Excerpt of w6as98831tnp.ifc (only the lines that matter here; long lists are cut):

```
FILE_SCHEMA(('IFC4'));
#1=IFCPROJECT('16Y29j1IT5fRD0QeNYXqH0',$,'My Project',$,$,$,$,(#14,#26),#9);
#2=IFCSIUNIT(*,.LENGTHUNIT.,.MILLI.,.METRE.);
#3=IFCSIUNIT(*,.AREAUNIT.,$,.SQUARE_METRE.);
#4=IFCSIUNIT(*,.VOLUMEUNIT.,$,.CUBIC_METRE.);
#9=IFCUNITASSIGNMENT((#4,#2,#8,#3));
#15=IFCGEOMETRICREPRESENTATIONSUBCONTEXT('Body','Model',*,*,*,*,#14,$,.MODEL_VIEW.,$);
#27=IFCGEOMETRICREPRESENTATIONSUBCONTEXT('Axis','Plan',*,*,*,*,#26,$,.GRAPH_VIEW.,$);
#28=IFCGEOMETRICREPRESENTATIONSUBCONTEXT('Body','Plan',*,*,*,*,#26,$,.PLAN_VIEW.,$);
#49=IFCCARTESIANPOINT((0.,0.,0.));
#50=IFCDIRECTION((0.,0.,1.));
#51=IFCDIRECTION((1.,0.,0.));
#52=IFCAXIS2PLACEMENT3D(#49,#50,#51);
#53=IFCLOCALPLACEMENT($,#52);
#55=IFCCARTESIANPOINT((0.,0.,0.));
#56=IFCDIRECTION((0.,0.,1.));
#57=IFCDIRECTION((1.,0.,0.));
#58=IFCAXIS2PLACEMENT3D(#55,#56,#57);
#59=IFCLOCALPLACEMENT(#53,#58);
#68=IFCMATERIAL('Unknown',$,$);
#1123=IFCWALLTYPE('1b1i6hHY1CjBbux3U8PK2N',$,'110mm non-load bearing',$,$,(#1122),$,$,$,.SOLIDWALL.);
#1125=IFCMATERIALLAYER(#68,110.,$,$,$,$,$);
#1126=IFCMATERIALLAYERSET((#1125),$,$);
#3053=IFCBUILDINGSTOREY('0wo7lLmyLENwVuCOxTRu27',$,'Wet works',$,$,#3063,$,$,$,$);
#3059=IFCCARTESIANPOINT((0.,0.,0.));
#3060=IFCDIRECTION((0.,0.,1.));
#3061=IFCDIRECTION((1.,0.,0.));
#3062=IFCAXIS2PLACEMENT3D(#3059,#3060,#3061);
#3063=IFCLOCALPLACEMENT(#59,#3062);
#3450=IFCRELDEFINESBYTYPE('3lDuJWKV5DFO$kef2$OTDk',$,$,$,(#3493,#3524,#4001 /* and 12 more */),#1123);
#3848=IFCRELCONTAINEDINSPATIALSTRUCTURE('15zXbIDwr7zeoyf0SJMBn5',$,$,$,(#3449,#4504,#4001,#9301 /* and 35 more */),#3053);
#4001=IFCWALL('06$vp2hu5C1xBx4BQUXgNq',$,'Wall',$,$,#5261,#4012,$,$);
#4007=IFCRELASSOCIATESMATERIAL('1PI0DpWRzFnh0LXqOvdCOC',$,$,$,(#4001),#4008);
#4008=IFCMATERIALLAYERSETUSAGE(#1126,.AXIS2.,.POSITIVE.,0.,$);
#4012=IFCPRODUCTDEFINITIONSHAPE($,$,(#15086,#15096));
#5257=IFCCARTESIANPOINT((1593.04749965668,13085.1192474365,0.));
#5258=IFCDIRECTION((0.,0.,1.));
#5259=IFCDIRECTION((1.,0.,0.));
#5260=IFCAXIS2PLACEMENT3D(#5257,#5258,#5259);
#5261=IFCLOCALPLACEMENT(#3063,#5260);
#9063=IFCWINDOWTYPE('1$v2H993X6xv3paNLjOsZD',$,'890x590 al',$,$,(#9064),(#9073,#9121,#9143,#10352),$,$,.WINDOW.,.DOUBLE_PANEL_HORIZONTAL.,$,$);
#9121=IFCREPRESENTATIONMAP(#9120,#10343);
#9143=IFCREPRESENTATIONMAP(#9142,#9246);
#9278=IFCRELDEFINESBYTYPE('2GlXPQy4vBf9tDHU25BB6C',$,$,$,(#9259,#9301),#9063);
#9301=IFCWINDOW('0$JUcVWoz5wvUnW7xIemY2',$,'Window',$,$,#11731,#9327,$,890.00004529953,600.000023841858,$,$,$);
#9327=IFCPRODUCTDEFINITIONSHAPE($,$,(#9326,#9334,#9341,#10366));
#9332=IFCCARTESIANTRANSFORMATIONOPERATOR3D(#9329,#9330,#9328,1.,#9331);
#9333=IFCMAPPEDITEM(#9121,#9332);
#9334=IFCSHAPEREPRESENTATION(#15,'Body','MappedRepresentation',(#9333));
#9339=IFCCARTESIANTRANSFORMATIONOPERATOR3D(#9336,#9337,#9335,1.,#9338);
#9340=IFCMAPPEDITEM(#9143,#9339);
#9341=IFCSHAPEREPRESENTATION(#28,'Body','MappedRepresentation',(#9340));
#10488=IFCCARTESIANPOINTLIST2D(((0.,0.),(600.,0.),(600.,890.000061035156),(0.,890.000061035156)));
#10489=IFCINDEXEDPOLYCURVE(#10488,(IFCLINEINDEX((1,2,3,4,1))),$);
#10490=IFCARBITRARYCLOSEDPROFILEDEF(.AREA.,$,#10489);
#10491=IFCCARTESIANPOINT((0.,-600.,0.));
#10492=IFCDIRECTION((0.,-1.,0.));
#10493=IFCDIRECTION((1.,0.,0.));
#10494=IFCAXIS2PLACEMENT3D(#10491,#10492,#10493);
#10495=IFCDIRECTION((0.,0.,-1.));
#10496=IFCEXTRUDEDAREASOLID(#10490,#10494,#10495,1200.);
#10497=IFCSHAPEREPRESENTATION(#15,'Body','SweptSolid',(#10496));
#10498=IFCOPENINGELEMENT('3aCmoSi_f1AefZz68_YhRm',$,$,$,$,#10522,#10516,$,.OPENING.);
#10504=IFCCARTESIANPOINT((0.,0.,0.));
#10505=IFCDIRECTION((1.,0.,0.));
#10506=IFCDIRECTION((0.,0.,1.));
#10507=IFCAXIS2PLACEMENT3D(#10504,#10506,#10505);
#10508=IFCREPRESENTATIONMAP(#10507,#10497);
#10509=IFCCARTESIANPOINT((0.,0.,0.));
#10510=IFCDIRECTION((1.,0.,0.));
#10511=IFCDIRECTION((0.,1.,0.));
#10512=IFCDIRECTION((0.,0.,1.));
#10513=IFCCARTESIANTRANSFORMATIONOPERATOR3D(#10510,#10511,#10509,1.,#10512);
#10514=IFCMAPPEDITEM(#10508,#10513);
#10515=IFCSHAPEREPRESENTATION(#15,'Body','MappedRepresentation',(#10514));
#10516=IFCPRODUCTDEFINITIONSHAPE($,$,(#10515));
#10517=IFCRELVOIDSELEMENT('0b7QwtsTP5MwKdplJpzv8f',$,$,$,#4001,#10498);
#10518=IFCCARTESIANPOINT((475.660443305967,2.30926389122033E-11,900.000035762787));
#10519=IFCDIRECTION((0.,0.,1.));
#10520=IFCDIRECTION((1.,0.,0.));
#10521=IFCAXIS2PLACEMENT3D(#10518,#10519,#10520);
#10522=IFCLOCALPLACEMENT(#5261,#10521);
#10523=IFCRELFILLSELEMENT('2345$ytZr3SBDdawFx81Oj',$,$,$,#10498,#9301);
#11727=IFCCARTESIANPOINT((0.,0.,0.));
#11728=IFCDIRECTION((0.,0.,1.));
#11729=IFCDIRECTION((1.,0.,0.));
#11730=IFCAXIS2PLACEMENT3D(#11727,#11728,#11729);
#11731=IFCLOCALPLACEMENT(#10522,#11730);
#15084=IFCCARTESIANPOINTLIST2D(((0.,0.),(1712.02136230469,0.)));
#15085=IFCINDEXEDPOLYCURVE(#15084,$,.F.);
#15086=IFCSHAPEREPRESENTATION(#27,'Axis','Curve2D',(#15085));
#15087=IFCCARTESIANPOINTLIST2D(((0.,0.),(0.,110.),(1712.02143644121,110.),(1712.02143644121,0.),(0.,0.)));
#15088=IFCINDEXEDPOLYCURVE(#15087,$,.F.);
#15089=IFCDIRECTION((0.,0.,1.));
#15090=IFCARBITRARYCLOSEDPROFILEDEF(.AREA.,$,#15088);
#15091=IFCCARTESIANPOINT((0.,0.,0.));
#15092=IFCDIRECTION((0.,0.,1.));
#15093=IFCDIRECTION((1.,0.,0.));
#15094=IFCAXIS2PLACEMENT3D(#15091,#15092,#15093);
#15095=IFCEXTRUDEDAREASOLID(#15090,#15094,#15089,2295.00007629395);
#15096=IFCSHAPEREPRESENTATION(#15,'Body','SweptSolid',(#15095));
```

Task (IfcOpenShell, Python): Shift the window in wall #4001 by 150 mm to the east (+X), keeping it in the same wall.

```python
import ifcopenshell
import ifcopenshell.api.geometry
import ifcopenshell.util.placement
import ifcopenshell.util.unit

model = ifcopenshell.open("w6as98831tnp.ifc")
unit_scale = ifcopenshell.util.unit.calculate_unit_scale(model)

window = model.by_guid("0$JUcVWoz5wvUnW7xIemY2")
opening = window.FillsVoids[0].RelatingOpeningElement
wall = opening.VoidsElements[0].RelatingBuildingElement

wall_matrix = ifcopenshell.util.placement.get_local_placement(wall.ObjectPlacement)
shift = wall_matrix[:3, 0] * 0.15 / unit_scale
before = ifcopenshell.util.placement.get_local_placement(window.ObjectPlacement)[:3, 3].copy()

# The window is placed relative to its opening, so it follows when the opening moves.
matrix = ifcopenshell.util.placement.get_local_placement(opening.ObjectPlacement)
matrix[:3, 3] += shift
ifcopenshell.api.geometry.edit_object_placement(
    model, product=opening, matrix=matrix, is_si=False, should_transform_children=True
)

after = ifcopenshell.util.placement.get_local_placement(window.ObjectPlacement)[:3, 3]
print("window moved by", (after - before).round(3) + 0.0)

model.write("w6as98831tnp_rev.ifc")
```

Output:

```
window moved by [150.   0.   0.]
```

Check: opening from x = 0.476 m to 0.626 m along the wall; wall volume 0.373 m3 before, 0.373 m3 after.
